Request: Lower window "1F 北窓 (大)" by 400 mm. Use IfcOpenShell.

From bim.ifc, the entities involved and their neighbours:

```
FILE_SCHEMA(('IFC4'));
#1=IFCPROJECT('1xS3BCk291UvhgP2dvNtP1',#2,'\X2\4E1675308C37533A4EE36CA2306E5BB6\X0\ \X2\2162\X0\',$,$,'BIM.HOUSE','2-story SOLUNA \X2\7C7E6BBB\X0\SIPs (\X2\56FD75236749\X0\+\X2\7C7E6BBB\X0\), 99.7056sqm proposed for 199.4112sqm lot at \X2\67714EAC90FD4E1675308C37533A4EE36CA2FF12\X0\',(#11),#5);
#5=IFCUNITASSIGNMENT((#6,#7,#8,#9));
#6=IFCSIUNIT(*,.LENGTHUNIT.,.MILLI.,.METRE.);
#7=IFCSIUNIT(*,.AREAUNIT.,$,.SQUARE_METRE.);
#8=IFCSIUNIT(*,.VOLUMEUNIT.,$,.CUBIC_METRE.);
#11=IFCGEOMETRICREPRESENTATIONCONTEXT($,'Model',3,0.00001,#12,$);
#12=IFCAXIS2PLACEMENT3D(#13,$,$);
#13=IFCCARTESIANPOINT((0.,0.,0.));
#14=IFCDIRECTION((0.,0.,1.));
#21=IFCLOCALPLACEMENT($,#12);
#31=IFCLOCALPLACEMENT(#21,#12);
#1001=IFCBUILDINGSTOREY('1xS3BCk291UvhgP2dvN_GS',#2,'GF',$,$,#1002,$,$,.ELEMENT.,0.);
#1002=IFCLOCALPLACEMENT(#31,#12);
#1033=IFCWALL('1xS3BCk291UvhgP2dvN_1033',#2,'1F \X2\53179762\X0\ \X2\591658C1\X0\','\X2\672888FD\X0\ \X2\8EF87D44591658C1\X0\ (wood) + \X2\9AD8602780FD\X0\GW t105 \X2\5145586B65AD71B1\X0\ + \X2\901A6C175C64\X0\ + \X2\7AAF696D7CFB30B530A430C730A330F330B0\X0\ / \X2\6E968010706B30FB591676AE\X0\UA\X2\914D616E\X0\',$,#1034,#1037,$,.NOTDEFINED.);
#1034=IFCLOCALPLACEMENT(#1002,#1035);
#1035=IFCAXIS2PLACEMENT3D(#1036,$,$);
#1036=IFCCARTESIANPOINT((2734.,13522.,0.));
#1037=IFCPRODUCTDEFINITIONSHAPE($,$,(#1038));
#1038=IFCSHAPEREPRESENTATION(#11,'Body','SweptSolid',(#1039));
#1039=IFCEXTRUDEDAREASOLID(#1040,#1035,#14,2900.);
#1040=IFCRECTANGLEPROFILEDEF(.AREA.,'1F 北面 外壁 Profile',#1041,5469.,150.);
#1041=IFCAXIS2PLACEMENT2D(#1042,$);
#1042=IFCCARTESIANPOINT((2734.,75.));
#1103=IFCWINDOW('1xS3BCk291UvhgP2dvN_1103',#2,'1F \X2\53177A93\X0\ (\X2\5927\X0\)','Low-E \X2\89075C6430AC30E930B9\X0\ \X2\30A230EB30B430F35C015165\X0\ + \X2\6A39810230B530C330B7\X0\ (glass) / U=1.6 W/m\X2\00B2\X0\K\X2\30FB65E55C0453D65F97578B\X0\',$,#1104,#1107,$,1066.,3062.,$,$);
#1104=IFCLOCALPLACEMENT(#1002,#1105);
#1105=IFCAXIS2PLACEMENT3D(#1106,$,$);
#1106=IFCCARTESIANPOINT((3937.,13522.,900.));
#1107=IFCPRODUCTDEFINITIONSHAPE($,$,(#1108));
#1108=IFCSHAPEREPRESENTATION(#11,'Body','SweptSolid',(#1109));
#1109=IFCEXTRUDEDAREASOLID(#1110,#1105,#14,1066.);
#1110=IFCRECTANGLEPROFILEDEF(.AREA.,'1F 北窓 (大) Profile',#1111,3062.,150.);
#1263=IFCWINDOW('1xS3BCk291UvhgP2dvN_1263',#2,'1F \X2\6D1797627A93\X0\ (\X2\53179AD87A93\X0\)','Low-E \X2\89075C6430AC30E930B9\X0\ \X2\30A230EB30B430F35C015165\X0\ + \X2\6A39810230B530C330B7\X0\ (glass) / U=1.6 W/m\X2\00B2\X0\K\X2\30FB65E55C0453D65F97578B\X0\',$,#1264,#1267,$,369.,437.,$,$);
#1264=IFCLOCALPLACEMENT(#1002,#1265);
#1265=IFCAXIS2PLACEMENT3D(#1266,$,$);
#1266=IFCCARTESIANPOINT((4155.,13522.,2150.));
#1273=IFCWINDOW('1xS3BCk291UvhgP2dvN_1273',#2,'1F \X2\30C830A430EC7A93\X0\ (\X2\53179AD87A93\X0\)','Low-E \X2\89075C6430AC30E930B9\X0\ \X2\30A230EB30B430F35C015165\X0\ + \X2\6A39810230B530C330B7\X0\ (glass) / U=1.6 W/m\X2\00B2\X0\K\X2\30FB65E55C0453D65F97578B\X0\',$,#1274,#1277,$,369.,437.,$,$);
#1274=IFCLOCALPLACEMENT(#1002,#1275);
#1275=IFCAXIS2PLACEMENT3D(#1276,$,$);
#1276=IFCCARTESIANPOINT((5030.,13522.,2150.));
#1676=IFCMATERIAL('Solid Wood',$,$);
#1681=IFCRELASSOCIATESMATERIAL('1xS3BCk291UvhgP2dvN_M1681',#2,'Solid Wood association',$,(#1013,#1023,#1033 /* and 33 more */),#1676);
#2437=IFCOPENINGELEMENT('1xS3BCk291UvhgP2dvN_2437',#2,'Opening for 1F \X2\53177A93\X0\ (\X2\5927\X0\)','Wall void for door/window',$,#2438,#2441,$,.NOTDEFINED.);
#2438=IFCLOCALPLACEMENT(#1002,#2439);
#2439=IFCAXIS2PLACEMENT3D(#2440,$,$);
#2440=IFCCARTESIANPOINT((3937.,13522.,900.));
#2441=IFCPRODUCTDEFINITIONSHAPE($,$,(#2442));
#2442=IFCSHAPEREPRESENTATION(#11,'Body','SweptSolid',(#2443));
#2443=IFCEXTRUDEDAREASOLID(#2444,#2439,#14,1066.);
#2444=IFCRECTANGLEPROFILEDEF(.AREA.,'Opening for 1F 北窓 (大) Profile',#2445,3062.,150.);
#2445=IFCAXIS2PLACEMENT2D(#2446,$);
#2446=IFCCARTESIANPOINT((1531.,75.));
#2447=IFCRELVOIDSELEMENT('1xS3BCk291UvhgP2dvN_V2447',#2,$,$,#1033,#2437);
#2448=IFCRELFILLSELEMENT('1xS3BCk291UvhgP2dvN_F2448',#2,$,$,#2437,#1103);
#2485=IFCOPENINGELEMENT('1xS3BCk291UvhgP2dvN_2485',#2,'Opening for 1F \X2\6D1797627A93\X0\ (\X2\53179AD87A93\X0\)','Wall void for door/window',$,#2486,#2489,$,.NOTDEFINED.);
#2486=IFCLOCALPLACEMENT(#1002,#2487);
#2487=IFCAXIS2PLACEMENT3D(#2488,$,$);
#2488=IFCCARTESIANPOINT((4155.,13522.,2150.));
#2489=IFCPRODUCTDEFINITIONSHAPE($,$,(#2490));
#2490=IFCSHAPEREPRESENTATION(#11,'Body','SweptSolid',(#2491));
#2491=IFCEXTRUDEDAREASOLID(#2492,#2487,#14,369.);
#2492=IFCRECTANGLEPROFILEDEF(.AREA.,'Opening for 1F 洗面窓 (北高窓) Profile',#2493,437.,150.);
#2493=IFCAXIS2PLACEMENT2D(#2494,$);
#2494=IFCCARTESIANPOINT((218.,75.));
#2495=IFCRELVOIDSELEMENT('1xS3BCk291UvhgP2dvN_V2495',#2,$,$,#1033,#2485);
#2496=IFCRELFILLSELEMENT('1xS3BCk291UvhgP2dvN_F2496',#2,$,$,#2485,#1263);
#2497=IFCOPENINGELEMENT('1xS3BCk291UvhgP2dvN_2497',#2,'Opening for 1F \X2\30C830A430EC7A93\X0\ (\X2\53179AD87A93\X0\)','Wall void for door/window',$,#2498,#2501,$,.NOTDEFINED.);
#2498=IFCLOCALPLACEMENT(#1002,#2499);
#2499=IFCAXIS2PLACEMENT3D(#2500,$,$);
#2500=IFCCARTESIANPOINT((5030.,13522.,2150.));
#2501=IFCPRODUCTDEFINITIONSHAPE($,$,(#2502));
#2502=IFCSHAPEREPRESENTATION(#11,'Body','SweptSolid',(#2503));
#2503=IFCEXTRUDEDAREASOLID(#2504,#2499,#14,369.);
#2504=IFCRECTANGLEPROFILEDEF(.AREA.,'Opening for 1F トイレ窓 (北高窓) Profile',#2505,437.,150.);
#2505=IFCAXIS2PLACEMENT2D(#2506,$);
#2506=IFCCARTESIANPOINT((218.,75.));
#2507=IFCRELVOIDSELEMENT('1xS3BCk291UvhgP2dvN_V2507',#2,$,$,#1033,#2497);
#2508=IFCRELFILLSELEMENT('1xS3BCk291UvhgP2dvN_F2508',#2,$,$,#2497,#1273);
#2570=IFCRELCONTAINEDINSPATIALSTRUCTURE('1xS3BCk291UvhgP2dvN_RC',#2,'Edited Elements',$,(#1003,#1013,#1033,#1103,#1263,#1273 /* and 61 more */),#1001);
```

```python
import numpy as np
import ifcopenshell
import ifcopenshell.api.geometry
import ifcopenshell.util.placement
import ifcopenshell.util.unit

model = ifcopenshell.open("bim.ifc")
unit_scale = ifcopenshell.util.unit.calculate_unit_scale(model)

window = model.by_guid("1xS3BCk291UvhgP2dvN_1103")
opening = window.FillsVoids[0].RelatingOpeningElement
dz = -0.4 / unit_scale

shift = np.array([0.0, 0.0, dz])
# The window is not placed relative to its opening, so move both.
for product in (opening, window):
    matrix = ifcopenshell.util.placement.get_local_placement(product.ObjectPlacement)
    matrix[:3, 3] += shift
    ifcopenshell.api.geometry.edit_object_placement(model, product=product, matrix=matrix, is_si=False)

print(f"moved by {dz * unit_scale:+.3f} m")

model.write("bim_rev.ifc")
```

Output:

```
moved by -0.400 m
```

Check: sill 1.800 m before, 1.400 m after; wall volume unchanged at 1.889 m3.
